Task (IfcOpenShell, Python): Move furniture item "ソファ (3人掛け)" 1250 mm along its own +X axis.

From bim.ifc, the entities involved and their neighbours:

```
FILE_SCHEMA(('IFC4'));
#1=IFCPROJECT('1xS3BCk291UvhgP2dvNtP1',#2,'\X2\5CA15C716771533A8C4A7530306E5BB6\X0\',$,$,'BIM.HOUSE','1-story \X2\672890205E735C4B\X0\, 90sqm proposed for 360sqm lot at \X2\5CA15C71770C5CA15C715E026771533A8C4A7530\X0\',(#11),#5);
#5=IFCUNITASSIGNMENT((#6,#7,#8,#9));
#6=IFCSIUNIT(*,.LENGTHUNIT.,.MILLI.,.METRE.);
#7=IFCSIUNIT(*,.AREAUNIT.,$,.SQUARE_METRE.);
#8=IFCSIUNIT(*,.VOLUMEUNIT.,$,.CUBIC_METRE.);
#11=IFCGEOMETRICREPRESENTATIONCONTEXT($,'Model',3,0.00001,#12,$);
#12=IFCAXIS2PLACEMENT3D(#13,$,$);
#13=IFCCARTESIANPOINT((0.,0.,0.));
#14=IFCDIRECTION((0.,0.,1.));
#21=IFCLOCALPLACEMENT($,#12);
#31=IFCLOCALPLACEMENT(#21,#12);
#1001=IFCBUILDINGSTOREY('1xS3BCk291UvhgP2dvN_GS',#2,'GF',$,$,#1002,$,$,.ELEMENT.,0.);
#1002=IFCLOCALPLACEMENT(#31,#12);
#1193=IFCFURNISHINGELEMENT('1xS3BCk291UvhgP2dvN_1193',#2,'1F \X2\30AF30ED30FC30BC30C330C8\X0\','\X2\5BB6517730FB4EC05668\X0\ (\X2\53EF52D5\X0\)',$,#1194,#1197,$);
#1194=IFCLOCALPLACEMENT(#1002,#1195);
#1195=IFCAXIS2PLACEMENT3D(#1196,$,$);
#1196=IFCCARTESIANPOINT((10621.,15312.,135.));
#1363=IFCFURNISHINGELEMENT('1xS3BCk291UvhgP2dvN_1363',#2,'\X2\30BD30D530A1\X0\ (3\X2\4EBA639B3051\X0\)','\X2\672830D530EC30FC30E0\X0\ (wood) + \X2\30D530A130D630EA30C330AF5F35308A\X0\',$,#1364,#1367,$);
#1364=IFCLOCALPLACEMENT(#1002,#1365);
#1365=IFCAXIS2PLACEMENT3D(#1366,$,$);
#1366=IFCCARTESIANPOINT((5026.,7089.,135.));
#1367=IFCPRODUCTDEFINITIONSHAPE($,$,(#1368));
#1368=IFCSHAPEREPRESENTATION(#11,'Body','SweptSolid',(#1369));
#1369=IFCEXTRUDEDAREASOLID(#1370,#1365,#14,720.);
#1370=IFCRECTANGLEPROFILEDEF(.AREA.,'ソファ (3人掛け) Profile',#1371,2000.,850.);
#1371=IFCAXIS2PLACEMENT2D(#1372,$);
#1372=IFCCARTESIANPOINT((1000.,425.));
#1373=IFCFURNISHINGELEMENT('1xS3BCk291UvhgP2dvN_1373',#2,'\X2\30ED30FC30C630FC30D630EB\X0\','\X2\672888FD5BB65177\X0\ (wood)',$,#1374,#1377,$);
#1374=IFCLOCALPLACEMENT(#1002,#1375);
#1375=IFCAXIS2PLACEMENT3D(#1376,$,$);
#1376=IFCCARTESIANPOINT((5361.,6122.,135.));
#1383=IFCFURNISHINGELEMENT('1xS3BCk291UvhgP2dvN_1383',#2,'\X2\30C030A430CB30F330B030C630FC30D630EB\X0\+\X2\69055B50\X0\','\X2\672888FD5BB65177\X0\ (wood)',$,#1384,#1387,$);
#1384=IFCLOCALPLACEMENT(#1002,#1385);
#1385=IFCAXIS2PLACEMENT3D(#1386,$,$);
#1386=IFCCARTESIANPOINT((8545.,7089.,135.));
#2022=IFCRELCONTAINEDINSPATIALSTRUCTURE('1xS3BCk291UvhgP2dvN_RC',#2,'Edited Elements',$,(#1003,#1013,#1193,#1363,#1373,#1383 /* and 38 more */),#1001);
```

```python
import ifcopenshell
import ifcopenshell.api.geometry
import ifcopenshell.util.placement

model = ifcopenshell.open("bim.ifc")

item = model.by_guid("1xS3BCk291UvhgP2dvN_1363")
matrix = ifcopenshell.util.placement.get_local_placement(item.ObjectPlacement)
matrix[:3, 3] += matrix[:3, 0] * 1250.0
ifcopenshell.api.geometry.edit_object_placement(model, product=item, matrix=matrix, is_si=False)

print(ifcopenshell.util.placement.get_local_placement(item.ObjectPlacement).round(3) + 0.0)

model.write("bim-out.ifc")
```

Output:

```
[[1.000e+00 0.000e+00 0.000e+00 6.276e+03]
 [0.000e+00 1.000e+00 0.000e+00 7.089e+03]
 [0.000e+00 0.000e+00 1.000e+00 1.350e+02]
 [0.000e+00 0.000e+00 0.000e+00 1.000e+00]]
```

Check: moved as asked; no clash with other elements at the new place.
